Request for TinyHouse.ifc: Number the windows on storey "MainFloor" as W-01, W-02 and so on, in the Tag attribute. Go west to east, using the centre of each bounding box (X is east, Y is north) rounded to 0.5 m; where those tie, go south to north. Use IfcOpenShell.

First a look at what the model holds.

```python
import ifcopenshell
import ifcopenshell.util.element
import ifcopenshell.util.placement

model = ifcopenshell.open("TinyHouse.ifc")
print(model.schema)
storey = next(s for s in model.by_type("IfcBuildingStorey") if s.Name == "MainFloor")
windows = [e for e in ifcopenshell.util.element.get_decomposition(storey) if e.is_a("IfcWindow")]
for e in sorted(windows, key=lambda e: e.id()):
    origin = ifcopenshell.util.placement.get_local_placement(e.ObjectPlacement)[:3, 3]
    print(e.id(), e.Tag, e.Name, origin.round(2) + 0.0, sep=" | ")
```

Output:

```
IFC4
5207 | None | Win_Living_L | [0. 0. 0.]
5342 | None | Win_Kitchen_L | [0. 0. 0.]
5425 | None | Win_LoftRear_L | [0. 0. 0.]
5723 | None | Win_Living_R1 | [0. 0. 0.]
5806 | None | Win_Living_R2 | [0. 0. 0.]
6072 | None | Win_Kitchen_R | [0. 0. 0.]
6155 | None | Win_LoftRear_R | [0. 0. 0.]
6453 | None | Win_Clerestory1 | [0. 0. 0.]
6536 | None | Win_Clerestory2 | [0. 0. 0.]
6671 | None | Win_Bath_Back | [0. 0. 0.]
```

```python
import ifcopenshell
import ifcopenshell.geom
import ifcopenshell.util.element
import ifcopenshell.util.shape

model = ifcopenshell.open("TinyHouse.ifc")
settings = ifcopenshell.geom.settings()
settings.set("use-world-coords", True)


def centre(element):
    shape = ifcopenshell.geom.create_shape(settings, element)
    return ifcopenshell.util.shape.get_bbox_centroid(shape.geometry)


storey = next(s for s in model.by_type("IfcBuildingStorey") if s.Name == "MainFloor")
windows = [e for e in ifcopenshell.util.element.get_decomposition(storey) if e.is_a("IfcWindow")]

# Insertion points can sit at a corner or the storey origin, so sort by the geometry (in metres).
centres = {e: centre(e) for e in windows}
windows.sort(key=lambda e: (round(centres[e][0] / 0.5), centres[e][1]))

for i, e in enumerate(windows, start=1):
    number = f"W-{i:02d}"
    e.Tag = number
    print(e.id(), number)

model.write("TinyHouse_updated.ifc")
```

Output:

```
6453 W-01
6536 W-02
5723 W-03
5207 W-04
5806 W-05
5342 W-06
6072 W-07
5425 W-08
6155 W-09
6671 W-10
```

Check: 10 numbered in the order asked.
